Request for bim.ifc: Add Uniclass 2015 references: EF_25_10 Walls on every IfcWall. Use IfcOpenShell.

First a look at what the model holds.

```python
import ifcopenshell

model = ifcopenshell.open("bim.ifc")
print(model.schema)
print("classifications:", [c.Name for c in model.by_type("IfcClassification")])
for ifc_class in ("IfcDoor", "IfcRoof", "IfcStair", "IfcWall", "IfcWindow"):
    print(ifc_class, len(model.by_type(ifc_class)))
```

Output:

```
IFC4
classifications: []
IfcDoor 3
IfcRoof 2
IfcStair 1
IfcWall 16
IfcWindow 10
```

```python
import ifcopenshell
import ifcopenshell.api.classification

model = ifcopenshell.open("bim.ifc")

system = ifcopenshell.api.classification.add_classification(model, classification="Uniclass 2015")

codes = {
    "IfcWall": ("EF_25_10", "Walls"),
}
for ifc_class, (code, name) in codes.items():
    products = model.by_type(ifc_class)
    ifcopenshell.api.classification.add_reference(
        model, products=products, classification=system, identification=code, name=name
    )
    print(code, len(products))

model.write("bim_updated.ifc")
```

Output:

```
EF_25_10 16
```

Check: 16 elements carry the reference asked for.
